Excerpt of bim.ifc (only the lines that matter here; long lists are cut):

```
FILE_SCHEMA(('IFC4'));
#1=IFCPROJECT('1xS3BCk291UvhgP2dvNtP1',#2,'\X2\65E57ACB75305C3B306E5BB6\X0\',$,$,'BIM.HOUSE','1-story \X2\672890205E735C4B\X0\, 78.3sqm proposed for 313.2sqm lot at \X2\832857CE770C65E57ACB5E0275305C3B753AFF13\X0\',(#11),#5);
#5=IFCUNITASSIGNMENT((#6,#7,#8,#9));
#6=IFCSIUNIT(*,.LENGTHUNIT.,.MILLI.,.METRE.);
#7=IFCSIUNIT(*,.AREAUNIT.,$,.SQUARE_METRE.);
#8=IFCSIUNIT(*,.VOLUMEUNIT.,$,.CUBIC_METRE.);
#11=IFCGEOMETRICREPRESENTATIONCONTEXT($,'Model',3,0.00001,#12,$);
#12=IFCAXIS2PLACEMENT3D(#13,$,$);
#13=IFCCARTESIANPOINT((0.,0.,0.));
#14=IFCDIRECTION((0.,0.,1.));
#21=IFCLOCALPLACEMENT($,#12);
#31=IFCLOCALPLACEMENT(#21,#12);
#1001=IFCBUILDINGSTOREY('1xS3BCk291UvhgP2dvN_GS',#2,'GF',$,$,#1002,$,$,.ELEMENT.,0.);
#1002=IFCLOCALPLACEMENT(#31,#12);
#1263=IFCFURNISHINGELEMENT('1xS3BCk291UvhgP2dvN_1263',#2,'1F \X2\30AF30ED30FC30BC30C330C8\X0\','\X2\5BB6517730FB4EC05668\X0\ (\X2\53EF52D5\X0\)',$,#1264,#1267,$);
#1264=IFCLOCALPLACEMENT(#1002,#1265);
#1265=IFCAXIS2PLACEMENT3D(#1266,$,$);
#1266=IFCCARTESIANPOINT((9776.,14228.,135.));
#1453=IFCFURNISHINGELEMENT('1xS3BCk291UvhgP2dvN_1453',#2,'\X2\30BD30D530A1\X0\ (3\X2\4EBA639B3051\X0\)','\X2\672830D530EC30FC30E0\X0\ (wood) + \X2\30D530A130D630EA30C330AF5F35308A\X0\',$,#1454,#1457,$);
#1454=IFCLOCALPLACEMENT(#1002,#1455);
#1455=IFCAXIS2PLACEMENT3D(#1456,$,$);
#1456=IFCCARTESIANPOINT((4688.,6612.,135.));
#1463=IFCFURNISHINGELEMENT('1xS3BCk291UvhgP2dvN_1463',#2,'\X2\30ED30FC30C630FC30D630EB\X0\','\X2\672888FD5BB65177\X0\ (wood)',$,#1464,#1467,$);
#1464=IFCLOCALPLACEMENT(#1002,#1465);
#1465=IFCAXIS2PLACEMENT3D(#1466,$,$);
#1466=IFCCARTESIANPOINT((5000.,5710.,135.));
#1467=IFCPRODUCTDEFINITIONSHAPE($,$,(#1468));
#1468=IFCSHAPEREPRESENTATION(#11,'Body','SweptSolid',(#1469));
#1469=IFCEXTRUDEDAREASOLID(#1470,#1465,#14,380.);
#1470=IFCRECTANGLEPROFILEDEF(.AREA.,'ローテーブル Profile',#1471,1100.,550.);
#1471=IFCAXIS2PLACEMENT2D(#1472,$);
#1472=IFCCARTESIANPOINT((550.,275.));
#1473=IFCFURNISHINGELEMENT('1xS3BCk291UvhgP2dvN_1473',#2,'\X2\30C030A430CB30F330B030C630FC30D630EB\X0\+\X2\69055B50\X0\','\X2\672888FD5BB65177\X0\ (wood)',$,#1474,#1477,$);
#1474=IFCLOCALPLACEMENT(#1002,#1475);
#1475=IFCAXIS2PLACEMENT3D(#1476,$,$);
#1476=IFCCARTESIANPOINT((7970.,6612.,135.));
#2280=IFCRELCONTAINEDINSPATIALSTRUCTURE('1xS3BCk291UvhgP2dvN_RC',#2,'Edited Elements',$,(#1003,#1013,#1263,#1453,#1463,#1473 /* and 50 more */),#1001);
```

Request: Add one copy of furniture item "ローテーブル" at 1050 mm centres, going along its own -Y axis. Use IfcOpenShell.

```python
import ifcopenshell
import ifcopenshell.api.geometry
import ifcopenshell.api.root
import ifcopenshell.util.element
import ifcopenshell.util.placement

model = ifcopenshell.open("bim.ifc")


def reuse_history(source, copy):
    """copy_class also copies each property set's owner history, people and application; keep the originals."""
    for rel in copy.IsDefinedBy:
        if rel.is_a("IfcRelDefinesByProperties") and (history := rel.RelatingPropertyDefinition.OwnerHistory):
            rel.RelatingPropertyDefinition.OwnerHistory = source.OwnerHistory
            ifcopenshell.util.element.remove_deep2(model, history)


source = model.by_id(1463)
base = ifcopenshell.util.placement.get_local_placement(source.ObjectPlacement)
step = -base[:3, 1] * 1050.0

for i in range(1, 2):
    copy = ifcopenshell.api.root.copy_class(model, product=source)
    copy.Representation = ifcopenshell.util.element.copy_deep(
        model, source.Representation, exclude=["IfcGeometricRepresentationContext", "IfcRepresentationMap"]
    )
    reuse_history(source, copy)
    matrix = base.copy()
    matrix[:3, 3] += i * step
    print("added at", matrix[:3, 3].round(3) + 0.0)
    ifcopenshell.api.geometry.edit_object_placement(model, product=copy, matrix=matrix, is_si=False)

model.write("bim_v2.ifc")
```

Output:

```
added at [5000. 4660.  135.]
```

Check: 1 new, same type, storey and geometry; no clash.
